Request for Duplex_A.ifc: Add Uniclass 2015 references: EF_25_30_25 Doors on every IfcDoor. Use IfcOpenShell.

First a look at what the model holds.

```python
import ifcopenshell

model = ifcopenshell.open("Duplex_A.ifc")
print(model.schema)
print("classifications:", [c.Name for c in model.by_type("IfcClassification")])
for ifc_class in ("IfcDoor", "IfcRoof", "IfcStair", "IfcWall", "IfcWindow"):
    print(ifc_class, len(model.by_type(ifc_class)))
```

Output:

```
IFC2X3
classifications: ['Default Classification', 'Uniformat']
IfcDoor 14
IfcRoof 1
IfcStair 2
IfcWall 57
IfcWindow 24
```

```python
import ifcopenshell
import ifcopenshell.api.classification

model = ifcopenshell.open("Duplex_A.ifc")

# IFC2X3 requires Source and Edition and has no link from the project to the system.
system = model.create_entity("IfcClassification", Source="NBS", Edition="2015", Name="Uniclass 2015")

codes = {
    "IfcDoor": ("EF_25_30_25", "Doors"),
}
for ifc_class, (code, name) in codes.items():
    products = model.by_type(ifc_class)
    ifcopenshell.api.classification.add_reference(
        model, products=products, classification=system, identification=code, name=name
    )
    print(code, len(products))

model.write("Duplex_A_edited.ifc")
```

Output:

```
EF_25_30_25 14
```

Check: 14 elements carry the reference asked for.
